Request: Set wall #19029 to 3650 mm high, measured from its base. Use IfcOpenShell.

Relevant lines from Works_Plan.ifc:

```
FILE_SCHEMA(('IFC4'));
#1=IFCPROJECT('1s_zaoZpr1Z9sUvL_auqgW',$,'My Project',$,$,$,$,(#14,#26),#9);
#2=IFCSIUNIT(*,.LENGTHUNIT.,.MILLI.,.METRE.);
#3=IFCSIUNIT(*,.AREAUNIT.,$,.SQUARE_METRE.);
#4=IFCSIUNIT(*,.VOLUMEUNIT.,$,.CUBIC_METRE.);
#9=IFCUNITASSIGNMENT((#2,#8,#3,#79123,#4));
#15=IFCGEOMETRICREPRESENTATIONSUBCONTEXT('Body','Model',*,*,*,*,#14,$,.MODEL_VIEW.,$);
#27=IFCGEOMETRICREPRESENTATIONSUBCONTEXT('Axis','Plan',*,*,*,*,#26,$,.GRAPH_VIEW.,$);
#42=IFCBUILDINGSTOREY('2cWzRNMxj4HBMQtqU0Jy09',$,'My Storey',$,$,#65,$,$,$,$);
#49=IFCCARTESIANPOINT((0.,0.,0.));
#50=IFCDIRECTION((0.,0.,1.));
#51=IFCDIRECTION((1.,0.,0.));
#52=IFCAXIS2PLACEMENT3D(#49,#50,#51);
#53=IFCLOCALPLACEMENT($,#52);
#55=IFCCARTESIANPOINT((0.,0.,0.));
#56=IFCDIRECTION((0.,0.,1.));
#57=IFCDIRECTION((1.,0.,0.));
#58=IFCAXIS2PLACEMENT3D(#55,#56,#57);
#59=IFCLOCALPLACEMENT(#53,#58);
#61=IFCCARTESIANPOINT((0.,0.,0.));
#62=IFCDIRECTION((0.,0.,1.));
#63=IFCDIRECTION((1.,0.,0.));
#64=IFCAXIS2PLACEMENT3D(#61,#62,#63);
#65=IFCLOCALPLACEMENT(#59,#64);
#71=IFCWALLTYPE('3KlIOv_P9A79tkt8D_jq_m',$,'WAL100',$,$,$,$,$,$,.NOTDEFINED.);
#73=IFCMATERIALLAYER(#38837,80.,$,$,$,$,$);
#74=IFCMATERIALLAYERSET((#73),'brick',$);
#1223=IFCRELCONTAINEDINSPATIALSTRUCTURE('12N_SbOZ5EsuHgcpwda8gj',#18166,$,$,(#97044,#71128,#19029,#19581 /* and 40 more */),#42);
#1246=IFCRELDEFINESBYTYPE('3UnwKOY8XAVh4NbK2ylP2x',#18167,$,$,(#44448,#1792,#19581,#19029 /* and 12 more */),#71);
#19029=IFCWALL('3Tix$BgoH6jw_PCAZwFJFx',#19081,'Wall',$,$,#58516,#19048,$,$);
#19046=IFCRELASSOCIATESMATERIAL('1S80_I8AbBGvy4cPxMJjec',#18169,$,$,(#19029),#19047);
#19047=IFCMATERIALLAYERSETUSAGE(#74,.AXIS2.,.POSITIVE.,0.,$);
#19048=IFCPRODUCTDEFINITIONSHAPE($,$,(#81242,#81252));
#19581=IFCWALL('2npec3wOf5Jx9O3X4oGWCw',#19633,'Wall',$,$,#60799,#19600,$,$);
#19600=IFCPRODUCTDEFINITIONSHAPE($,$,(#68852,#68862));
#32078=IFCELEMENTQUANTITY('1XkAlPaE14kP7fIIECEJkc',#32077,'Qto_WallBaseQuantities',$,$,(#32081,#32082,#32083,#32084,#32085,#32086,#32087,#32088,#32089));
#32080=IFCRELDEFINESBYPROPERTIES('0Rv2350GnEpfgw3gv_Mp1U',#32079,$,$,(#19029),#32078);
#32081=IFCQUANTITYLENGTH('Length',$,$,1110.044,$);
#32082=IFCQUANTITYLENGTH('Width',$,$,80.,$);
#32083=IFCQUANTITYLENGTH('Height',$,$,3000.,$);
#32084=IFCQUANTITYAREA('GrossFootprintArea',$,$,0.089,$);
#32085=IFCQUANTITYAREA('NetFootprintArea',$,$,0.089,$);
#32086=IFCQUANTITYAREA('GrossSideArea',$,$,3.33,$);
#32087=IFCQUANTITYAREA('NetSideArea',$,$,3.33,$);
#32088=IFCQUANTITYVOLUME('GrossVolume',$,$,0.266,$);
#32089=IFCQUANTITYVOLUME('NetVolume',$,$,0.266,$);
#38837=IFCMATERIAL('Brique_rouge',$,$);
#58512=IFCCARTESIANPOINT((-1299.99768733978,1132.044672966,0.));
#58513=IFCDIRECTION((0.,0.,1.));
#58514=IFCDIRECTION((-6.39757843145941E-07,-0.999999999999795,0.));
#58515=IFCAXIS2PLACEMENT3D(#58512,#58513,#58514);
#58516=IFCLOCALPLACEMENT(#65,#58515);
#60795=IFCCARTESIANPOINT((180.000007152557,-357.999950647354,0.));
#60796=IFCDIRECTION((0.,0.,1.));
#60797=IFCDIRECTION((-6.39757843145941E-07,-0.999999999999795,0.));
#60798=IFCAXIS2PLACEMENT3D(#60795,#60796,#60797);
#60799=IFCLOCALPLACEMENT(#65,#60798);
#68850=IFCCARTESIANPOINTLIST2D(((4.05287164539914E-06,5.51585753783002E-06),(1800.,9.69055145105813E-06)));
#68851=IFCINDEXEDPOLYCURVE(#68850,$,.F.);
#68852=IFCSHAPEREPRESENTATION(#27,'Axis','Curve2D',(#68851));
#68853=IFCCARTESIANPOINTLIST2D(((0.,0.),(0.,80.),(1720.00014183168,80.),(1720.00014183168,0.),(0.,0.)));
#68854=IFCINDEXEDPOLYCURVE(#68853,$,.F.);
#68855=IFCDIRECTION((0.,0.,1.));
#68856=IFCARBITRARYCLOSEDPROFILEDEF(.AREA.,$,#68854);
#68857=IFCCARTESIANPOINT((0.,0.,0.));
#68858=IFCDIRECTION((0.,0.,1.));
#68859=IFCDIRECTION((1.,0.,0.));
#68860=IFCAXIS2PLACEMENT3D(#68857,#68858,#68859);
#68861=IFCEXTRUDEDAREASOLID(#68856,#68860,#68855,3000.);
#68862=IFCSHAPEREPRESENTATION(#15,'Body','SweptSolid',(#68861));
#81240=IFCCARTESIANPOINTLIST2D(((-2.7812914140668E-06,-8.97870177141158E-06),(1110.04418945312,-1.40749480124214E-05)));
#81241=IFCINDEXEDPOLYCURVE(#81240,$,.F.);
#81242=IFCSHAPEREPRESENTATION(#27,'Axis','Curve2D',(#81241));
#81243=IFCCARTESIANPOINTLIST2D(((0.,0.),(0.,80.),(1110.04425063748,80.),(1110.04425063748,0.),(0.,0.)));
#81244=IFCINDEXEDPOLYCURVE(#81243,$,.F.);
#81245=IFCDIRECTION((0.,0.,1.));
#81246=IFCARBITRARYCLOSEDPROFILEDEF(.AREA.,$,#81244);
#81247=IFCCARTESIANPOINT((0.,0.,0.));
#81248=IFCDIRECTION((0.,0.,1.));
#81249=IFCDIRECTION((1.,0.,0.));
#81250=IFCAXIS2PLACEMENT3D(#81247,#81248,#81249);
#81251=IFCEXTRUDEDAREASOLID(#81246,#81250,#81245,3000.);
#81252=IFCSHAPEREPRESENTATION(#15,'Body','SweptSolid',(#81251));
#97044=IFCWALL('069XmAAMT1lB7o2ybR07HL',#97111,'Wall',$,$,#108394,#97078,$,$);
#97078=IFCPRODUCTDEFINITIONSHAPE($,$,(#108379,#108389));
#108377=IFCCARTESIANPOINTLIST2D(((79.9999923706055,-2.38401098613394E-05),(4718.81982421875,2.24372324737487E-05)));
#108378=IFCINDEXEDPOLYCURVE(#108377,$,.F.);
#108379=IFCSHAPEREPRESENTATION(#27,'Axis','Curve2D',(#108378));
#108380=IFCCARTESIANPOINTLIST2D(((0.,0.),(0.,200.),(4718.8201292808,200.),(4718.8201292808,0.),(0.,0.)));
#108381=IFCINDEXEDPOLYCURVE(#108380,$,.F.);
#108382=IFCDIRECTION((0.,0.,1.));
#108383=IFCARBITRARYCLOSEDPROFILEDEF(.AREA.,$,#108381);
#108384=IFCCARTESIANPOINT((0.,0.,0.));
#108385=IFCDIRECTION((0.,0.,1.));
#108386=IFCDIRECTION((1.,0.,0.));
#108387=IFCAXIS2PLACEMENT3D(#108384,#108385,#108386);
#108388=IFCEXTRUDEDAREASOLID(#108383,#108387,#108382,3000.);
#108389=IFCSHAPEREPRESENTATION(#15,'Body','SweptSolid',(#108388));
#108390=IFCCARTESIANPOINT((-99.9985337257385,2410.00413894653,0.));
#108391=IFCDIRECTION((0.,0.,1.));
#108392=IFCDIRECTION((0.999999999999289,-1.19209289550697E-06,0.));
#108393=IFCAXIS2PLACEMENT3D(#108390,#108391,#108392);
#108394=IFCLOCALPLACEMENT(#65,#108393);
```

```python
import ifcopenshell
import ifcopenshell.api.pset
import ifcopenshell.geom
import ifcopenshell.util.element
import ifcopenshell.util.representation
import ifcopenshell.util.shape
import ifcopenshell.util.unit

model = ifcopenshell.open("Works_Plan.ifc")
unit_scale = ifcopenshell.util.unit.calculate_unit_scale(model)
area_scale = ifcopenshell.util.unit.calculate_unit_scale(model, "AREAUNIT")
volume_scale = ifcopenshell.util.unit.calculate_unit_scale(model, "VOLUMEUNIT")
settings = ifcopenshell.geom.settings()


def volume(element):
    """Net volume in cubic metres, openings subtracted."""
    shape = ifcopenshell.geom.create_shape(settings, element)
    return ifcopenshell.util.shape.get_volume(shape.geometry)


wall = model.by_guid("3Tix$BgoH6jw_PCAZwFJFx")
before = volume(wall)

body = ifcopenshell.util.representation.get_representation(wall, "Model", "Body")
solid = body.Items[0]
old_height = solid.Depth
solid.Depth = 3650.0
after = volume(wall)
thickness = 0.08  # wall thickness in metres

# Update the stored height, areas and volumes.
qto = model.by_id(ifcopenshell.util.element.get_pset(wall, "Qto_WallBaseQuantities", should_inherit=False)["id"])
ifcopenshell.api.pset.edit_qto(model, qto=qto, properties={
    "Height": solid.Depth,
    "GrossSideArea": ifcopenshell.util.element.get_pset(wall, "Qto_WallBaseQuantities", "GrossSideArea") * solid.Depth / old_height,
    "NetSideArea": after / thickness / area_scale,
    "GrossVolume": ifcopenshell.util.element.get_pset(wall, "Qto_WallBaseQuantities", "GrossVolume") * solid.Depth / old_height,
    "NetVolume": after / volume_scale,
})

print(f"height {old_height:g} -> {solid.Depth:g}, volume {before:.3f} -> {after:.3f} m3")

model.write("Works_Plan_v2.ifc")
```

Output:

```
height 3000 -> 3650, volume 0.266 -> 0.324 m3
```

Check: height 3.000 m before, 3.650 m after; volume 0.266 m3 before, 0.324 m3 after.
